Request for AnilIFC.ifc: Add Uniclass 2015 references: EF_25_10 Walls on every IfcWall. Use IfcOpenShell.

First a look at what the model holds.

```python
import ifcopenshell

model = ifcopenshell.open("AnilIFC.ifc")
print(model.schema)
print("classifications:", [c.Name for c in model.by_type("IfcClassification")])
for ifc_class in ("IfcDoor", "IfcRoof", "IfcStair", "IfcWall", "IfcWindow"):
    print(ifc_class, len(model.by_type(ifc_class)))
```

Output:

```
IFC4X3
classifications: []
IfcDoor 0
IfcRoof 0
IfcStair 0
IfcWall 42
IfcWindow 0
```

```python
import ifcopenshell
import ifcopenshell.api.classification

model = ifcopenshell.open("AnilIFC.ifc")

system = ifcopenshell.api.classification.add_classification(model, classification="Uniclass 2015")

codes = {
    "IfcWall": ("EF_25_10", "Walls"),
}
for ifc_class, (code, name) in codes.items():
    products = model.by_type(ifc_class)
    ifcopenshell.api.classification.add_reference(
        model, products=products, classification=system, identification=code, name=name
    )
    print(code, len(products))

model.write("AnilIFC_updated.ifc")
```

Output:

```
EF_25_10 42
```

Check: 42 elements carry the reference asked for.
